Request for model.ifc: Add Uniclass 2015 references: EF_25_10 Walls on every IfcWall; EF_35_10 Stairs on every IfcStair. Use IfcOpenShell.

First a look at what the model holds.

```python
import ifcopenshell

model = ifcopenshell.open("model.ifc")
print(model.schema)
print("classifications:", [c.Name for c in model.by_type("IfcClassification")])
for ifc_class in ("IfcDoor", "IfcRoof", "IfcStair", "IfcWall", "IfcWindow"):
    print(ifc_class, len(model.by_type(ifc_class)))
```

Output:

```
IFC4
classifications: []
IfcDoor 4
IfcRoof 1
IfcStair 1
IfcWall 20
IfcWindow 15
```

```python
import ifcopenshell
import ifcopenshell.api.classification

model = ifcopenshell.open("model.ifc")

system = ifcopenshell.api.classification.add_classification(model, classification="Uniclass 2015")

codes = {
    "IfcWall": ("EF_25_10", "Walls"),
    "IfcStair": ("EF_35_10", "Stairs"),
}
for ifc_class, (code, name) in codes.items():
    products = model.by_type(ifc_class)
    ifcopenshell.api.classification.add_reference(
        model, products=products, classification=system, identification=code, name=name
    )
    print(code, len(products))

model.write("model_updated.ifc")
```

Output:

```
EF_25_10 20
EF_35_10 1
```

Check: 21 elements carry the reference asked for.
